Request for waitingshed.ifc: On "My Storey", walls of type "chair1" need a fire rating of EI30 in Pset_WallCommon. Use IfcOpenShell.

First a look at what the model holds.

```python
import ifcopenshell
import ifcopenshell.util.element

model = ifcopenshell.open("waitingshed.ifc")
print(model.schema)
storey = next(s for s in model.by_type("IfcBuildingStorey") if s.Name == "My Storey")
walls = [e for e in ifcopenshell.util.element.get_decomposition(storey) if e.is_a("IfcWall")]
seen = {}
for e in walls:
    element_type = ifcopenshell.util.element.get_type(e)
    key = (element_type.Name if element_type != e and element_type else None, ifcopenshell.util.element.get_pset(e, "Pset_WallCommon", "FireRating"))
    seen[key] = seen.get(key, 0) + 1
for (name, value), count in sorted(seen.items(), key=str):
    print(count, "x", name, "|", value)
```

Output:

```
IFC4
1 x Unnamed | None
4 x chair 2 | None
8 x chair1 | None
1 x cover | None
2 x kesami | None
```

```python
import ifcopenshell
import ifcopenshell.api.pset
import ifcopenshell.util.element

model = ifcopenshell.open("waitingshed.ifc")

storey = next(s for s in model.by_type("IfcBuildingStorey") if s.Name == "My Storey")
walls = [e for e in ifcopenshell.util.element.get_decomposition(storey) if e.is_a("IfcWall")]

count = 0
for e in walls:
    element_type = ifcopenshell.util.element.get_type(e)
    if element_type in (None, e) or element_type.Name != "chair1":
        continue
    # add_pset returns the element's existing set when there is one.
    pset = ifcopenshell.api.pset.add_pset(model, product=e, name="Pset_WallCommon")
    ifcopenshell.api.pset.edit_pset(model, pset=pset, properties={"FireRating": "EI30"})
    count += 1

print(count, "walls updated")

model.write("waitingshed-out.ifc")
```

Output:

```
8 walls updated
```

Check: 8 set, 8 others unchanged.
